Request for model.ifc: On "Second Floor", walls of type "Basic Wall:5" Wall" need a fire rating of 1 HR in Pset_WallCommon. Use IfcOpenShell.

First a look at what the model holds.

```python
import ifcopenshell
import ifcopenshell.util.element

model = ifcopenshell.open("model.ifc")
print(model.schema)
storey = next(s for s in model.by_type("IfcBuildingStorey") if s.Name == "Second Floor")
walls = [e for e in ifcopenshell.util.element.get_decomposition(storey) if e.is_a("IfcWall")]
seen = {}
for e in walls:
    element_type = ifcopenshell.util.element.get_type(e)
    key = (element_type.Name if element_type != e and element_type else None, ifcopenshell.util.element.get_pset(e, "Pset_WallCommon", "FireRating"))
    seen[key] = seen.get(key, 0) + 1
for (name, value), count in sorted(seen.items(), key=str):
    print(count, "x", name, "|", value)
```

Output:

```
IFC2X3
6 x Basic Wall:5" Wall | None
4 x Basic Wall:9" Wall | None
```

```python
import ifcopenshell
import ifcopenshell.api.pset
import ifcopenshell.util.element

model = ifcopenshell.open("model.ifc")

storey = next(s for s in model.by_type("IfcBuildingStorey") if s.Name == "Second Floor")
walls = [e for e in ifcopenshell.util.element.get_decomposition(storey) if e.is_a("IfcWall")]

count = 0
for e in walls:
    element_type = ifcopenshell.util.element.get_type(e)
    if element_type in (None, e) or element_type.Name != 'Basic Wall:5" Wall':
        continue
    # add_pset returns the element's existing set when there is one.
    pset = ifcopenshell.api.pset.add_pset(model, product=e, name="Pset_WallCommon")
    ifcopenshell.api.pset.edit_pset(model, pset=pset, properties={"FireRating": "1 HR"})
    count += 1

print(count, "walls updated")

model.write("model_edited.ifc")
```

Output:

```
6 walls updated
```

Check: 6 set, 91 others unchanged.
